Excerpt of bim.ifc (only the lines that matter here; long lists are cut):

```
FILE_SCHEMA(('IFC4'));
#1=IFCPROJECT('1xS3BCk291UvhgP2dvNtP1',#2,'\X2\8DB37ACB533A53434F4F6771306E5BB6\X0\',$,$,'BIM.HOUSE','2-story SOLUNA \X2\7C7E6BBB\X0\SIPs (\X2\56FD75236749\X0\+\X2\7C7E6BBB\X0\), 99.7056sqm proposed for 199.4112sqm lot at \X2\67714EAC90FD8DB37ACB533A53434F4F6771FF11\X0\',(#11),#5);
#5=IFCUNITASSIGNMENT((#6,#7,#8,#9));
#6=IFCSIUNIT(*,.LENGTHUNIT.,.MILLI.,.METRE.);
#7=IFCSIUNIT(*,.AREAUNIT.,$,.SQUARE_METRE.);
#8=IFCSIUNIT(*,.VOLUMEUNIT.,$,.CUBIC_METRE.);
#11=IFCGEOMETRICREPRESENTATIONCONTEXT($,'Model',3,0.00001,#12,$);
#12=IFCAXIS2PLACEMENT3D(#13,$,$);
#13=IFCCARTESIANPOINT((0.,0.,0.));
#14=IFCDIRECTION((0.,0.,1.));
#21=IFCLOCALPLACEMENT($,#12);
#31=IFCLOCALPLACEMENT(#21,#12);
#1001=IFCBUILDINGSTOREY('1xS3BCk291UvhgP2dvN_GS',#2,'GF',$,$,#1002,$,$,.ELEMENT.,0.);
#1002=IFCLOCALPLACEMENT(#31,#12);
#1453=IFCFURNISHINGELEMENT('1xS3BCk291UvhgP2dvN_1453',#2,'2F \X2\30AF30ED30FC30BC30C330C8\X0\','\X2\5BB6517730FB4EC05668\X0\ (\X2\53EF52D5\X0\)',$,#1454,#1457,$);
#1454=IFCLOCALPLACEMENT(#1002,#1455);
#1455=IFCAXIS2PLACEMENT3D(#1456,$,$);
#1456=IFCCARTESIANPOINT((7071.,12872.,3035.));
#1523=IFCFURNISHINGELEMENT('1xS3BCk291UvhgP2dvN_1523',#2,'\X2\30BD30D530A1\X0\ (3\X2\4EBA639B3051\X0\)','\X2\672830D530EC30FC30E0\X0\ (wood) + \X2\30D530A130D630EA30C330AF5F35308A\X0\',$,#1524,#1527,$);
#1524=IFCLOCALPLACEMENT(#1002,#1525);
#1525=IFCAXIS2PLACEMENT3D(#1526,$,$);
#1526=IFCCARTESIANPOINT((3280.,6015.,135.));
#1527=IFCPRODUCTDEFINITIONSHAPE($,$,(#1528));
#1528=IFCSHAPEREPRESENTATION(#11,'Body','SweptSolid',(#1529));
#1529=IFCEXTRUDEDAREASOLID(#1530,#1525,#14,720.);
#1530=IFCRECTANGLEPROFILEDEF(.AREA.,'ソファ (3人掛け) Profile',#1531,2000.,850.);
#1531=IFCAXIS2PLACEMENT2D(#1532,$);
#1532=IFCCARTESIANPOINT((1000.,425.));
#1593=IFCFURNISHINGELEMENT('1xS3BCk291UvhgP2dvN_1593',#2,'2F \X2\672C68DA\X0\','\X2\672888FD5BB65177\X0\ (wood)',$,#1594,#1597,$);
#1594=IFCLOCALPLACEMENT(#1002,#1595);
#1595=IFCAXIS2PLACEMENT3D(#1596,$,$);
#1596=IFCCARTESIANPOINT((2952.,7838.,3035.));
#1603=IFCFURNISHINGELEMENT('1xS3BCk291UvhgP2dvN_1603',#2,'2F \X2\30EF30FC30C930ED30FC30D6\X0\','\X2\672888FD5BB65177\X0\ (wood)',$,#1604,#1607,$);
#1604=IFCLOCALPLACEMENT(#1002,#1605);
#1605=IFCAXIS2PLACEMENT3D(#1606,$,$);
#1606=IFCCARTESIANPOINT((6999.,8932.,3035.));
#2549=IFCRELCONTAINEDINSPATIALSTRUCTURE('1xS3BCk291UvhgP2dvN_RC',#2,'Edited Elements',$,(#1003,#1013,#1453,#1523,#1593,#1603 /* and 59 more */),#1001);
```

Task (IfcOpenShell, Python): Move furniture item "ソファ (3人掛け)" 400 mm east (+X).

```python
import ifcopenshell
import ifcopenshell.api.geometry
import ifcopenshell.util.placement
import ifcopenshell.util.unit

model = ifcopenshell.open("bim.ifc")
unit_scale = ifcopenshell.util.unit.calculate_unit_scale(model)

item = model.by_id(1523)
matrix = ifcopenshell.util.placement.get_local_placement(item.ObjectPlacement)
matrix[0, 3] += 0.4 / unit_scale
ifcopenshell.api.geometry.edit_object_placement(model, product=item, matrix=matrix, is_si=False)

print(ifcopenshell.util.placement.get_local_placement(item.ObjectPlacement).round(3) + 0.0)

model.write("bim_v2.ifc")
```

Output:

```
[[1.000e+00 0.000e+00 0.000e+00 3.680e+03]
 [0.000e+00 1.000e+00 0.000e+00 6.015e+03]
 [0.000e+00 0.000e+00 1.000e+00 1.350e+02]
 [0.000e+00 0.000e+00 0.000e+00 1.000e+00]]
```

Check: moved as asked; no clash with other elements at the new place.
